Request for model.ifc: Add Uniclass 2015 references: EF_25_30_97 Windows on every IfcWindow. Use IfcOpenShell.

First a look at what the model holds.

```python
import ifcopenshell

model = ifcopenshell.open("model.ifc")
print(model.schema)
print("classifications:", [c.Name for c in model.by_type("IfcClassification")])
for ifc_class in ("IfcDoor", "IfcRoof", "IfcStair", "IfcWall", "IfcWindow"):
    print(ifc_class, len(model.by_type(ifc_class)))
```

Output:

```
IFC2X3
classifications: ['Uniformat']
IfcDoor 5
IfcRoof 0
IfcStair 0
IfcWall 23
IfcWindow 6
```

```python
import ifcopenshell
import ifcopenshell.api.classification

model = ifcopenshell.open("model.ifc")

# IFC2X3 requires Source and Edition and has no link from the project to the system.
system = model.create_entity("IfcClassification", Source="NBS", Edition="2015", Name="Uniclass 2015")

codes = {
    "IfcWindow": ("EF_25_30_97", "Windows"),
}
for ifc_class, (code, name) in codes.items():
    products = model.by_type(ifc_class)
    ifcopenshell.api.classification.add_reference(
        model, products=products, classification=system, identification=code, name=name
    )
    print(code, len(products))

model.write("model_edited.ifc")
```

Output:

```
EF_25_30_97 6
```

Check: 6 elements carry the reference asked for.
